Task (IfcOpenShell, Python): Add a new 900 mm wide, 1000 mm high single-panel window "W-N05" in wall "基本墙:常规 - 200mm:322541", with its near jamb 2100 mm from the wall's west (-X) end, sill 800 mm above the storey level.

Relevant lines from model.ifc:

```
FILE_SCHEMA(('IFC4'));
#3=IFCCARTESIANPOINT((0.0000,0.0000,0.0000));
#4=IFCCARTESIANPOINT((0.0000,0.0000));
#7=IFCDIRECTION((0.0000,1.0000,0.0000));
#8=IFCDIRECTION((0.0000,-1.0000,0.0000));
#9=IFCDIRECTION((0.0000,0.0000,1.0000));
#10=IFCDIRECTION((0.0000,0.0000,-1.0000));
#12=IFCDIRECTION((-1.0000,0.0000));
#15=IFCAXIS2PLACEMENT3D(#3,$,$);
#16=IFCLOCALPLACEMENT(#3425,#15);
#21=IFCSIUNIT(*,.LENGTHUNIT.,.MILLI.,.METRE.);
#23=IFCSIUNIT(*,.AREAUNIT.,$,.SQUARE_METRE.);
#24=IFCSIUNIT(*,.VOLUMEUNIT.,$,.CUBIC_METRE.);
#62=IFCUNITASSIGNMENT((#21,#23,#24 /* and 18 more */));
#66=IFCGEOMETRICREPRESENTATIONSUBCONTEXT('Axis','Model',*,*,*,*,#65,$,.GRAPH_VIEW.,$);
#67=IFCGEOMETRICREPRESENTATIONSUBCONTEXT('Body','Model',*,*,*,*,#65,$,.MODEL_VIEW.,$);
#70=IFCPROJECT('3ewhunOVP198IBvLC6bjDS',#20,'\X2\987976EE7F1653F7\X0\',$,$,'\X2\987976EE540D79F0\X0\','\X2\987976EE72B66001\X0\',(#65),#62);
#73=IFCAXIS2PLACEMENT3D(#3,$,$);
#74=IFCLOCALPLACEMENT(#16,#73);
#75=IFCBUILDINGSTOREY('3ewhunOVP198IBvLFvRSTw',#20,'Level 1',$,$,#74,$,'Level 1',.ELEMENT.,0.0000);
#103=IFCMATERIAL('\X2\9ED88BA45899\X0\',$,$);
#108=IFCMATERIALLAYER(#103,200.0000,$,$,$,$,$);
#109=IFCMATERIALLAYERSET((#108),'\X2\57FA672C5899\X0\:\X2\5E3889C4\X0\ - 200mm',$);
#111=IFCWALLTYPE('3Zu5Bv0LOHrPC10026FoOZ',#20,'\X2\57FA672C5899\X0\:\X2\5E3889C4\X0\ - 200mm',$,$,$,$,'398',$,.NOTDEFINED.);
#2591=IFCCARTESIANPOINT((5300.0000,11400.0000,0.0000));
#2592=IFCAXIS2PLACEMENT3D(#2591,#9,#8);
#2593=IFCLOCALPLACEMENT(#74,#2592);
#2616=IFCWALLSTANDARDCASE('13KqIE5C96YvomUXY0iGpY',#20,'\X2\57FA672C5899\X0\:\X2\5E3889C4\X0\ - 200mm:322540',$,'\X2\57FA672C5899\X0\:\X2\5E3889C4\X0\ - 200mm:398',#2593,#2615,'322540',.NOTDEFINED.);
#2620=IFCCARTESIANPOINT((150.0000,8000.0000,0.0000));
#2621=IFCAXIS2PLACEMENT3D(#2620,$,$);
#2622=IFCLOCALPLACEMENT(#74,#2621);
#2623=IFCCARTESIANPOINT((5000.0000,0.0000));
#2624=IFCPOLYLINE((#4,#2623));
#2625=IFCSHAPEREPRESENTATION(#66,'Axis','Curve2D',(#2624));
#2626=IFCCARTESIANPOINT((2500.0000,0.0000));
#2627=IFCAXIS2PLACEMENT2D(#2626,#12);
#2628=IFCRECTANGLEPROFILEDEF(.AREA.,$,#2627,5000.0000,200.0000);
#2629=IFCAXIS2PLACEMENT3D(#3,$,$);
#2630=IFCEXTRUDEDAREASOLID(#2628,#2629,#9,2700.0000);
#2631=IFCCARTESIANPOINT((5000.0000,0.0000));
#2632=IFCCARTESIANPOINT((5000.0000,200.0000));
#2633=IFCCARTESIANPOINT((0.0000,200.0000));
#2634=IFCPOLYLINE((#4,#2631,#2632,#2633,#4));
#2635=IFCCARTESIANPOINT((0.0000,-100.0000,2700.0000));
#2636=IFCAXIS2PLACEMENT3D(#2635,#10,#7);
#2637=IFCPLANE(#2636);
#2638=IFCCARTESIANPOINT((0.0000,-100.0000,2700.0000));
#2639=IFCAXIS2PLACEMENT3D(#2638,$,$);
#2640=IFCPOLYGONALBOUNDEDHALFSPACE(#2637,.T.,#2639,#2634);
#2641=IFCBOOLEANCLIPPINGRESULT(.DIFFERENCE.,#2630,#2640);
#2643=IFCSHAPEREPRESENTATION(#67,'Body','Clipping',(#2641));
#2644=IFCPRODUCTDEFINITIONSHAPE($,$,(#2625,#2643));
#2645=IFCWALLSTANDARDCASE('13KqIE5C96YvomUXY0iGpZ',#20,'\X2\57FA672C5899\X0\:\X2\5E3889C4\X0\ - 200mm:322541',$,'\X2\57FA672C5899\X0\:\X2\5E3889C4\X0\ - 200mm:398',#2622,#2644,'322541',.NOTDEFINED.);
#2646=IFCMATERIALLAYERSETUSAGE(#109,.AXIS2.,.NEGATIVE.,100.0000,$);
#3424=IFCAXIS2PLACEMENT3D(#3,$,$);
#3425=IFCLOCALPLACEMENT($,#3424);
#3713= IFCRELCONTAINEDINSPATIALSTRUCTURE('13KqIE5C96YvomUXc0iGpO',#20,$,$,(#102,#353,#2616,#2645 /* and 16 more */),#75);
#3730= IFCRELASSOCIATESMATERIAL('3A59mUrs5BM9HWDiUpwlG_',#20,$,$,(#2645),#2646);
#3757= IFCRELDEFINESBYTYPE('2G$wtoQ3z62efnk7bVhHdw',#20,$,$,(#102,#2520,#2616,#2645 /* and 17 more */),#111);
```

```python
import numpy as np
import ifcopenshell
import ifcopenshell.api.feature
import ifcopenshell.api.geometry
import ifcopenshell.api.root
import ifcopenshell.api.spatial
import ifcopenshell.geom
import ifcopenshell.util.element
import ifcopenshell.util.placement
import ifcopenshell.util.representation
import ifcopenshell.util.shape
import ifcopenshell.util.unit

model = ifcopenshell.open("model.ifc")
unit_scale = ifcopenshell.util.unit.calculate_unit_scale(model)
settings = ifcopenshell.geom.settings()


def volume(element):
    """Net volume in cubic metres, openings subtracted."""
    shape = ifcopenshell.geom.create_shape(settings, element)
    return ifcopenshell.util.shape.get_volume(shape.geometry)


wall = model.by_id(2645)
storey = ifcopenshell.util.element.get_container(wall, ifc_class="IfcBuildingStorey")
context = ifcopenshell.util.representation.get_context(model, "Model", "Body", "MODEL_VIEW")
before = volume(wall)

width, height, from_end, sill = 0.9, 1, 2.1, 0.8  # metres

# The wall runs along its own X axis, and the end named is its -X end.
wall_shape = ifcopenshell.geom.create_shape(settings, wall)
x, y, z = ifcopenshell.util.shape.get_vertices(wall_shape.geometry).T
start = x.min() + from_end
face, thickness = float(y.min()), float(y.max() - y.min())
wall_matrix = ifcopenshell.util.placement.get_local_placement(wall.ObjectPlacement)
level = ifcopenshell.util.placement.get_local_placement(storey.ObjectPlacement)[2, 3]


def in_wall(x, y):
    """Placement at x, y metres in the wall's axes, at sill height."""
    matrix = wall_matrix.copy()
    matrix[:, 3] = wall_matrix @ np.array([x / unit_scale, y / unit_scale, 0.0, 1.0])
    matrix[2, 3] = level + sill / unit_scale
    return matrix


# Opening: a box that overshoots both wall faces by 50 mm.
opening = ifcopenshell.api.root.create_entity(model, ifc_class="IfcOpeningElement", predefined_type="OPENING")
box = ifcopenshell.api.geometry.add_wall_representation(
    model, context=context, length=width, height=height, thickness=thickness + 0.1
)
ifcopenshell.api.geometry.assign_representation(model, product=opening, representation=box)
ifcopenshell.api.geometry.edit_object_placement(model, product=opening, matrix=in_wall(start, face - 0.05), is_si=False)
ifcopenshell.api.feature.add_feature(model, feature=opening, element=wall)

window = ifcopenshell.api.root.create_entity(model, ifc_class="IfcWindow", name="W-N05", predefined_type="WINDOW")
window.OverallWidth, window.OverallHeight = width / unit_scale, height / unit_scale
window.PartitioningType = "SINGLE_PANEL"
body = ifcopenshell.api.geometry.add_window_representation(
    model,
    context=context,
    overall_width=window.OverallWidth,
    overall_height=window.OverallHeight,
    partition_type="SINGLE_PANEL",
)
ifcopenshell.api.geometry.assign_representation(model, product=window, representation=body)
ifcopenshell.api.spatial.assign_container(model, products=[window], relating_structure=storey)
ifcopenshell.api.feature.add_filling(model, opening=opening, element=window)

# Centre the window in the wall's thickness.
ifcopenshell.api.geometry.edit_object_placement(model, product=window, matrix=in_wall(start, face), is_si=False)
window_shape = ifcopenshell.geom.create_shape(settings, window)
depth = ifcopenshell.util.shape.get_vertices(window_shape.geometry)[:, 1]
offset = face + thickness / 2 - (depth.min() + depth.max()) / 2
ifcopenshell.api.geometry.edit_object_placement(model, product=window, matrix=in_wall(start, offset), is_si=False)

after = volume(wall)

print(f"wall volume {before:.3f} -> {after:.3f} m3")

model.write("model_v2.ifc")
```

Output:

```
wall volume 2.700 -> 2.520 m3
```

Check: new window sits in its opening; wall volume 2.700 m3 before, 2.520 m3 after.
